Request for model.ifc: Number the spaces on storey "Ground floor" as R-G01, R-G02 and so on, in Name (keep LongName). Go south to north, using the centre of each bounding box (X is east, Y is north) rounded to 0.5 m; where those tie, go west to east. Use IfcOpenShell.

First a look at what the model holds.

```python
import ifcopenshell
import ifcopenshell.util.element
import ifcopenshell.util.placement

model = ifcopenshell.open("model.ifc")
print(model.schema)
storey = next(s for s in model.by_type("IfcBuildingStorey") if s.Name == "Ground floor")
spaces = [e for e in ifcopenshell.util.element.get_decomposition(storey) if e.is_a("IfcSpace")]
for e in sorted(spaces, key=lambda e: e.id()):
    origin = ifcopenshell.util.placement.get_local_placement(e.ObjectPlacement)[:3, 3]
    print(e.id(), e.Name, e.LongName, origin.round(2) + 0.0, sep=" | ")
```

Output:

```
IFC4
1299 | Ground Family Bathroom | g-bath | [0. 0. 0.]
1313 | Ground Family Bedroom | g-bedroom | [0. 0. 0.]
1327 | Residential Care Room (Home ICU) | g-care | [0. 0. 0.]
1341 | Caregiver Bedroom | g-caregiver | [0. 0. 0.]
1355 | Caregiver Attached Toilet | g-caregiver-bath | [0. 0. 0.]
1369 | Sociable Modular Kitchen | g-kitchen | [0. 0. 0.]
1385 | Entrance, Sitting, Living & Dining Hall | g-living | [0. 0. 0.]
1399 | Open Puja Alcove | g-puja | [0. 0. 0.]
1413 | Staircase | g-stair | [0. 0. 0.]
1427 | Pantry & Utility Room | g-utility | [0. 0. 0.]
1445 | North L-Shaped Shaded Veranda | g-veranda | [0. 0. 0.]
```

```python
import ifcopenshell
import ifcopenshell.geom
import ifcopenshell.util.element
import ifcopenshell.util.shape

model = ifcopenshell.open("model.ifc")
settings = ifcopenshell.geom.settings()
settings.set("use-world-coords", True)


def centre(element):
    shape = ifcopenshell.geom.create_shape(settings, element)
    return ifcopenshell.util.shape.get_bbox_centroid(shape.geometry)


storey = next(s for s in model.by_type("IfcBuildingStorey") if s.Name == "Ground floor")
spaces = [e for e in ifcopenshell.util.element.get_decomposition(storey) if e.is_a("IfcSpace")]

# Insertion points can sit at a corner or the storey origin, so sort by the geometry (in metres).
centres = {e: centre(e) for e in spaces}
spaces.sort(key=lambda e: (round(centres[e][1] / 0.5), centres[e][0]))

for i, e in enumerate(spaces, start=1):
    number = f"R-G{i:02d}"
    e.Name = number
    print(e.id(), number)

model.write("model_edited.ifc")
```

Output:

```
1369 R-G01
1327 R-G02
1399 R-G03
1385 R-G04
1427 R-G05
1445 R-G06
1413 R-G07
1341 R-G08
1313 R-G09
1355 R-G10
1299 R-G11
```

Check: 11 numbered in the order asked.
